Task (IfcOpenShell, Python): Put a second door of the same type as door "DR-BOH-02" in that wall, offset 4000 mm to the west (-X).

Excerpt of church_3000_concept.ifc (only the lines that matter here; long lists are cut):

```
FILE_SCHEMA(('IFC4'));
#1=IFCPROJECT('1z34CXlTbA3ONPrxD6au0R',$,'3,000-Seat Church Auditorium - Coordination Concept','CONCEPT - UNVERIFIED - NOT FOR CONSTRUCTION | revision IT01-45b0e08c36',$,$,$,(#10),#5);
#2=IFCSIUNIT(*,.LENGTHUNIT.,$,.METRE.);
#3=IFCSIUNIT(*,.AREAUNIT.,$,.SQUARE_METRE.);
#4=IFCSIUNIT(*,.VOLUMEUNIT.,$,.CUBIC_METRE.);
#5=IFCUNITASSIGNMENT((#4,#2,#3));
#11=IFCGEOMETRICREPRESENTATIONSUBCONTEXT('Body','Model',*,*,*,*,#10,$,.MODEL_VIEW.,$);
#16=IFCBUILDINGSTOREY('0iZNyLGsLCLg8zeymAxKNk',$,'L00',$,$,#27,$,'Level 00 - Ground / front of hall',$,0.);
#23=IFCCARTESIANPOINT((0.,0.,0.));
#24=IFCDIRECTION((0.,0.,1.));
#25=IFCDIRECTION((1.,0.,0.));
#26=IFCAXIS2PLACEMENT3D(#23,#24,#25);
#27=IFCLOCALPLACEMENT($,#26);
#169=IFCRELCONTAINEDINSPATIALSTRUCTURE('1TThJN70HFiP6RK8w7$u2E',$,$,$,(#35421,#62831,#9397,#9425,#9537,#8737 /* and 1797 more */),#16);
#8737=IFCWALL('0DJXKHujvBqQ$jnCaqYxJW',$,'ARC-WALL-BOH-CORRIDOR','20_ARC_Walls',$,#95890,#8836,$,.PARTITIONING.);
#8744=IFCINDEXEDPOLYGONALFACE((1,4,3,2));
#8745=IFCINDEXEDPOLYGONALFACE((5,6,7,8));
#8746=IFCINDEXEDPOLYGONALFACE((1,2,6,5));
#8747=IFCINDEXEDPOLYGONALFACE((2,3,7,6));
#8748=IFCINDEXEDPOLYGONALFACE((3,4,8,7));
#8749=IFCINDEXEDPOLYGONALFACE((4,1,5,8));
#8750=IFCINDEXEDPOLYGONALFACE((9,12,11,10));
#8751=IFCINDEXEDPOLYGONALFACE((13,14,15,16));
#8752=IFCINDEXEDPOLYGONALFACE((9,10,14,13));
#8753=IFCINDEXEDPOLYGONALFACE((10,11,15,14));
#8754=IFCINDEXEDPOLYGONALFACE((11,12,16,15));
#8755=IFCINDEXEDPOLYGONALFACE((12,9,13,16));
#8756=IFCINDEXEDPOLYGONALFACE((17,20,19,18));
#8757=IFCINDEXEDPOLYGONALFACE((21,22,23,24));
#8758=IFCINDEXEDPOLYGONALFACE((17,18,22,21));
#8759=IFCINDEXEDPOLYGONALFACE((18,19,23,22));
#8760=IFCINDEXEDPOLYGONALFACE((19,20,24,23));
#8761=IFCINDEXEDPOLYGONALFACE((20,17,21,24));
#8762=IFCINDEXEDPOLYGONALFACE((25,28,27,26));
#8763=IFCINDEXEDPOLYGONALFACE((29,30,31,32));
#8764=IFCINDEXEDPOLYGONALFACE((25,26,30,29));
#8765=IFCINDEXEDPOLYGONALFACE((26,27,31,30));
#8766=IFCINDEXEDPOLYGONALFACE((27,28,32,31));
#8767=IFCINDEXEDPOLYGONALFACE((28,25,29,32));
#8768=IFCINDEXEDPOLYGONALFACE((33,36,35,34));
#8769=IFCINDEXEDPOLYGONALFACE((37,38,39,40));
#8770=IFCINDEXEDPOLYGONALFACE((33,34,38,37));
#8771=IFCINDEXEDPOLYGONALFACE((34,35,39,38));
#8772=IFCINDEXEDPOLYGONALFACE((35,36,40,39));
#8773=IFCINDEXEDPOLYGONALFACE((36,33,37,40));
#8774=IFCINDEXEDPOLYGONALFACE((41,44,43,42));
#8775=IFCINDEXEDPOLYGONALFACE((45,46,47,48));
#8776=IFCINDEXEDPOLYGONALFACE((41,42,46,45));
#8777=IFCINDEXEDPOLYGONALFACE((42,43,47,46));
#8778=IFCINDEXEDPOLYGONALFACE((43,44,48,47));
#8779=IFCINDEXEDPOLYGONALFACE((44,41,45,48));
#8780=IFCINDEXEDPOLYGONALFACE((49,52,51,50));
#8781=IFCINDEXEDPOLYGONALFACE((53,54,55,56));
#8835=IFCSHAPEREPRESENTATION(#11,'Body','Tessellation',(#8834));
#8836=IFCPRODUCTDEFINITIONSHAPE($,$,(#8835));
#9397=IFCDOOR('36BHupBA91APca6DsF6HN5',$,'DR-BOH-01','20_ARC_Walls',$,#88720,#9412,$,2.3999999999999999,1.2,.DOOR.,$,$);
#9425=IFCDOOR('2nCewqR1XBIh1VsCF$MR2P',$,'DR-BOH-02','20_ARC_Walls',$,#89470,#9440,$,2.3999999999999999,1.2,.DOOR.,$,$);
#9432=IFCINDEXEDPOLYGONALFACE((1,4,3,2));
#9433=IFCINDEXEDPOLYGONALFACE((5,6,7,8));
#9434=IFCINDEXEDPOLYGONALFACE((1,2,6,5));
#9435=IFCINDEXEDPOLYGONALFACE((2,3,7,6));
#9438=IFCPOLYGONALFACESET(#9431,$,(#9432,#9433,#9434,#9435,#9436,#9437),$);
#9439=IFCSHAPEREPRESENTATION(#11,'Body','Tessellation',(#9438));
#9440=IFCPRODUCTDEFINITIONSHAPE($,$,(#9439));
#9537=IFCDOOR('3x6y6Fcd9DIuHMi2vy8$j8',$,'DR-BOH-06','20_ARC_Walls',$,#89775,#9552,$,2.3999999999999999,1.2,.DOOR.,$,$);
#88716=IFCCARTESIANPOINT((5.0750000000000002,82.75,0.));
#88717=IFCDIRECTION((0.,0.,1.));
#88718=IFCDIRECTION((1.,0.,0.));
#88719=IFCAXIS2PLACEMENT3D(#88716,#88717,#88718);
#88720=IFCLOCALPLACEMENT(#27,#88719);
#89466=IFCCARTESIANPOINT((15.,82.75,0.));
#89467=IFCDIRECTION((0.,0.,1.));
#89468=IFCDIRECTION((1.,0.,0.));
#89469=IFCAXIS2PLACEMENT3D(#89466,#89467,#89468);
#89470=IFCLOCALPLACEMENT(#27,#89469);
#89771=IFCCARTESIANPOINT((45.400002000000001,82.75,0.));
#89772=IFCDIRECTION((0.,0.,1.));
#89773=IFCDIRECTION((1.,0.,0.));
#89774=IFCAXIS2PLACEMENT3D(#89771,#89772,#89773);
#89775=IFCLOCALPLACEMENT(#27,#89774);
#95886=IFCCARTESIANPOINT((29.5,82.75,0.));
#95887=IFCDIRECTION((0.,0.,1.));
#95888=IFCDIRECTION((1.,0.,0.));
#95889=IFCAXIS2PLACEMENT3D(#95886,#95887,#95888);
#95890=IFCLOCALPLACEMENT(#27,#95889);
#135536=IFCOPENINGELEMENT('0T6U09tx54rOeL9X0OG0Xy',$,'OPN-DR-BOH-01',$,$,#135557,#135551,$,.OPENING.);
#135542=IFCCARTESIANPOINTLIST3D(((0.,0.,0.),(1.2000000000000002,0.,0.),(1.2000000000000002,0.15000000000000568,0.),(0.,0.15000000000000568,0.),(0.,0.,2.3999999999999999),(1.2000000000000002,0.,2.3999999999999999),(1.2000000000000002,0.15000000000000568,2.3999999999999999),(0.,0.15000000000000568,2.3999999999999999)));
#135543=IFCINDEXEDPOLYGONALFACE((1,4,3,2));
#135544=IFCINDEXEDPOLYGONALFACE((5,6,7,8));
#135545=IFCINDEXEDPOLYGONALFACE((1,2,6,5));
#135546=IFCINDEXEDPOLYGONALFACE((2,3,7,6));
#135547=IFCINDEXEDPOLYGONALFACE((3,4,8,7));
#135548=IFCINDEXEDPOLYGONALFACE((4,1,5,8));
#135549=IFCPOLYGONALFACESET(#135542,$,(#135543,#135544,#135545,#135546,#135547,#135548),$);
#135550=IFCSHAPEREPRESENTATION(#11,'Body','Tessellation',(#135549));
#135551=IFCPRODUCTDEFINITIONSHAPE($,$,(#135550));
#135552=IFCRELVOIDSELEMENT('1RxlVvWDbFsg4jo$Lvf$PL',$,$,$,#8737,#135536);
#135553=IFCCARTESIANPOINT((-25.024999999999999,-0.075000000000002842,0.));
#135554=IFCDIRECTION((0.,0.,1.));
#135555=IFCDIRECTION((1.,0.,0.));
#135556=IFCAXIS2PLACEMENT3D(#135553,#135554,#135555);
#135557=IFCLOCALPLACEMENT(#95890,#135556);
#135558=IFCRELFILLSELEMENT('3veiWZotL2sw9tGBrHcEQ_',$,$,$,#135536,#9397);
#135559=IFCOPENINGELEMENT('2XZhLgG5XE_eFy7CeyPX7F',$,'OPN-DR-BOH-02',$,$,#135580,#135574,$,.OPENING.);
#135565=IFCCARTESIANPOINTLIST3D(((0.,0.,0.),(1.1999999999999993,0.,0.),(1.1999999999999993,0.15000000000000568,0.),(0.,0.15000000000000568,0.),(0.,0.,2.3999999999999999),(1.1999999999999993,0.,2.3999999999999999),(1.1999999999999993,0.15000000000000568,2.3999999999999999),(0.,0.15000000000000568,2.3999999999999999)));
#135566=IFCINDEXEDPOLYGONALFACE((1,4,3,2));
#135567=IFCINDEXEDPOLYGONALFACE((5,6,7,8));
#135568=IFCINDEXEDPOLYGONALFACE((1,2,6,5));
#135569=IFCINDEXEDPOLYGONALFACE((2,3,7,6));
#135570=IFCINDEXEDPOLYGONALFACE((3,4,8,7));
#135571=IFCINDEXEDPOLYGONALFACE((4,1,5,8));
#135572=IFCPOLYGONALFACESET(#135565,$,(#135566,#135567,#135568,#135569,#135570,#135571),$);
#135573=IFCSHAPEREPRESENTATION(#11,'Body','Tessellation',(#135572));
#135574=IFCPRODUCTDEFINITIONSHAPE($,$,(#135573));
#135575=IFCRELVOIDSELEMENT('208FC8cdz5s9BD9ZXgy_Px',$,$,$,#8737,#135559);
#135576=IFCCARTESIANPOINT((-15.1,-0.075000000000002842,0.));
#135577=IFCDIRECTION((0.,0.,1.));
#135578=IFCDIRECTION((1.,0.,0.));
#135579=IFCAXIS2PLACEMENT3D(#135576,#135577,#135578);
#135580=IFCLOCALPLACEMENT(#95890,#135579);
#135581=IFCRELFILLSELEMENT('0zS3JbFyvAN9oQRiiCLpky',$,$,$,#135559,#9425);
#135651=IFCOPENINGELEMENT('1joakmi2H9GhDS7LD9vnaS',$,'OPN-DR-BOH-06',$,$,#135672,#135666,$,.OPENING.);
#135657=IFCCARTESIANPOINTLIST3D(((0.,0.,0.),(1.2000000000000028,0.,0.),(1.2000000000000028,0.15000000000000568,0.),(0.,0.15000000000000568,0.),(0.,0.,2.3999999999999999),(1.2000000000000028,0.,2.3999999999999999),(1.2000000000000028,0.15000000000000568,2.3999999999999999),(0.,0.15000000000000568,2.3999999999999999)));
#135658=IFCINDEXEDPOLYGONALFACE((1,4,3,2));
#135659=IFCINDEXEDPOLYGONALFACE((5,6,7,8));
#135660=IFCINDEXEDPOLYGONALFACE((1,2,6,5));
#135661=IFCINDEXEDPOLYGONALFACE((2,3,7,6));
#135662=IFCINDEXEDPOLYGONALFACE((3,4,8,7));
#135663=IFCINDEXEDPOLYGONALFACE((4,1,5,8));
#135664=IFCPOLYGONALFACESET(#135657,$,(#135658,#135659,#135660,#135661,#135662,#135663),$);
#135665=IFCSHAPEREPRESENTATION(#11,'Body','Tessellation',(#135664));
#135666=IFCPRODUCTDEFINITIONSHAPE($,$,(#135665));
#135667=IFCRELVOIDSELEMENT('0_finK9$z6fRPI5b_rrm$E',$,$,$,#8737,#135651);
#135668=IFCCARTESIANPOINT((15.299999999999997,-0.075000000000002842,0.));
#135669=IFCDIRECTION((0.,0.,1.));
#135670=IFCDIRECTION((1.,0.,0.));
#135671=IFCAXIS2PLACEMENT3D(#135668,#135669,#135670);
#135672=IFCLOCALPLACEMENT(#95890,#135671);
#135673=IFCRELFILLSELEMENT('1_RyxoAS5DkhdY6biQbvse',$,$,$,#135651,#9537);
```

```python
import ifcopenshell
import ifcopenshell.api.feature
import ifcopenshell.api.geometry
import ifcopenshell.api.root
import ifcopenshell.geom
import ifcopenshell.util.element
import ifcopenshell.util.placement
import ifcopenshell.util.shape
import ifcopenshell.util.unit

model = ifcopenshell.open("church_3000_concept.ifc")
unit_scale = ifcopenshell.util.unit.calculate_unit_scale(model)
settings = ifcopenshell.geom.settings()


def volume(element):
    """Net volume in cubic metres, openings subtracted."""
    shape = ifcopenshell.geom.create_shape(settings, element)
    return ifcopenshell.util.shape.get_volume(shape.geometry)


door = model.by_guid("2nCewqR1XBIh1VsCF$MR2P")
opening = door.FillsVoids[0].RelatingOpeningElement
wall = opening.VoidsElements[0].RelatingBuildingElement
before = volume(wall)
shift = ifcopenshell.util.placement.get_local_placement(wall.ObjectPlacement)[:3, 0] * -4 / unit_scale

# copy_class copies the void relationship, type, container and properties, but no geometry.
new_opening = ifcopenshell.api.root.copy_class(model, product=opening)
new_opening.Representation = ifcopenshell.util.element.copy_deep(
    model, opening.Representation, exclude=["IfcGeometricRepresentationContext", "IfcRepresentationMap"]
)
new_door = ifcopenshell.api.root.copy_class(model, product=door)
new_door.Representation = ifcopenshell.util.element.copy_deep(
    model, door.Representation, exclude=["IfcGeometricRepresentationContext", "IfcRepresentationMap"]
)
ifcopenshell.api.feature.add_filling(model, opening=new_opening, element=new_door)

for old, new in ((opening, new_opening), (door, new_door)):
    matrix = ifcopenshell.util.placement.get_local_placement(old.ObjectPlacement)
    matrix[:3, 3] += shift
    ifcopenshell.api.geometry.edit_object_placement(model, product=new, matrix=matrix, is_si=False)

after = volume(wall)

print(f"wall volume {before:.3f} -> {after:.3f} m3")

model.write("church_3000_concept_v2.ifc")
```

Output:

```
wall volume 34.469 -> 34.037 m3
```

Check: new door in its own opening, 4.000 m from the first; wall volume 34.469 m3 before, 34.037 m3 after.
